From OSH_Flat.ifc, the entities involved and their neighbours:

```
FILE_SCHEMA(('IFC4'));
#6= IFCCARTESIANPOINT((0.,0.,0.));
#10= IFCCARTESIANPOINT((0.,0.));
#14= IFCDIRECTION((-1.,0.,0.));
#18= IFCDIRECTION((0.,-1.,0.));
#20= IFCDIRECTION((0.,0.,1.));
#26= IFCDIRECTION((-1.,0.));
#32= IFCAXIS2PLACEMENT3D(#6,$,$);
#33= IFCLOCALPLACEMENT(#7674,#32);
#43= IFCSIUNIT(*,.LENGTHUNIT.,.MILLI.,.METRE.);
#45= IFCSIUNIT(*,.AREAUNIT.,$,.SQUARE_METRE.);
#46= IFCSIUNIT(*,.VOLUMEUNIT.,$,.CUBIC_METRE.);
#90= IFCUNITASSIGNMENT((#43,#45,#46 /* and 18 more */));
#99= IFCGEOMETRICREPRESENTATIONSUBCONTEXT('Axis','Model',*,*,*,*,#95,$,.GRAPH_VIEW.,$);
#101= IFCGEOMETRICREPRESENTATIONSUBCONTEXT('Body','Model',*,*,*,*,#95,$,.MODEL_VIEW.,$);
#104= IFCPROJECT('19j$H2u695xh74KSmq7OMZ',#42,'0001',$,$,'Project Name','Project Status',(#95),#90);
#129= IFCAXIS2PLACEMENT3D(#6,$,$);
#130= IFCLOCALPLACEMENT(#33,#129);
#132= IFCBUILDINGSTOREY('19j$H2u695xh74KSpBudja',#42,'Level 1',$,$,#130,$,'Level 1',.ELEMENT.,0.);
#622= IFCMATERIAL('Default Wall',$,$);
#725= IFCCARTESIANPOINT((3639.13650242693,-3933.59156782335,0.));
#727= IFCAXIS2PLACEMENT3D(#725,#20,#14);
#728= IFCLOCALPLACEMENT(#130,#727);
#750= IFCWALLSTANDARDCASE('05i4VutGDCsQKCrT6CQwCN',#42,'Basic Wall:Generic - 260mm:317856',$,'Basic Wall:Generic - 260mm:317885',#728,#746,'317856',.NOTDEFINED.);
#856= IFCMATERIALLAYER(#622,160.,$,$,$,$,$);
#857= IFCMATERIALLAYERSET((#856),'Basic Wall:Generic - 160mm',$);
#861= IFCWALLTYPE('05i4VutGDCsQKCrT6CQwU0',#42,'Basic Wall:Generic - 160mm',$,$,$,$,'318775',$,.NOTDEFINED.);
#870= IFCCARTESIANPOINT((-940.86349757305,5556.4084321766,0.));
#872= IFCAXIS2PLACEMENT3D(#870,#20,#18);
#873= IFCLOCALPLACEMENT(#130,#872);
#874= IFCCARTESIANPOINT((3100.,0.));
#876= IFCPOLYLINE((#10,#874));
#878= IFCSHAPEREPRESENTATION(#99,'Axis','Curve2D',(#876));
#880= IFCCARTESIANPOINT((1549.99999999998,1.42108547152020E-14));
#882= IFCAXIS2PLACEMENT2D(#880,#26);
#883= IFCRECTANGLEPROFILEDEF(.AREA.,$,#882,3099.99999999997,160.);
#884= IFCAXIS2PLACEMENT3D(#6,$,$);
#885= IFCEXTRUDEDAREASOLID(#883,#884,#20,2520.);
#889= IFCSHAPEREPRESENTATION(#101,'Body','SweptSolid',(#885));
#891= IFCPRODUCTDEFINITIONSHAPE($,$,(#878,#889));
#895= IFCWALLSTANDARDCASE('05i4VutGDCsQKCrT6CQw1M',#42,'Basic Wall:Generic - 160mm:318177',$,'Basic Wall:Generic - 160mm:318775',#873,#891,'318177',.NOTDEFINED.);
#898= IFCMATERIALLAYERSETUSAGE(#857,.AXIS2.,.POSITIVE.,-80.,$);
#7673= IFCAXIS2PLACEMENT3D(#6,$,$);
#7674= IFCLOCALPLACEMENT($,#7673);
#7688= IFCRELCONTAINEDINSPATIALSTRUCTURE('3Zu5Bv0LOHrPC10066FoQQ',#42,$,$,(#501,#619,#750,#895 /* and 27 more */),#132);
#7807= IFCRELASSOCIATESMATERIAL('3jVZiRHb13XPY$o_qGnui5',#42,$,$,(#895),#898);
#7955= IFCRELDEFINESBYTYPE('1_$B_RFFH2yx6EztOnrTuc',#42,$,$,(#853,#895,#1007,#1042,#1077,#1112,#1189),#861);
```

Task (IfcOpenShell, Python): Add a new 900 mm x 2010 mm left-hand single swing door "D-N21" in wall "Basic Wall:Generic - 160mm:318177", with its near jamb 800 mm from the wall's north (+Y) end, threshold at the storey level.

```python
import numpy as np
import ifcopenshell
import ifcopenshell.api.feature
import ifcopenshell.api.geometry
import ifcopenshell.api.root
import ifcopenshell.api.spatial
import ifcopenshell.geom
import ifcopenshell.util.element
import ifcopenshell.util.placement
import ifcopenshell.util.representation
import ifcopenshell.util.shape
import ifcopenshell.util.unit

model = ifcopenshell.open("OSH_Flat.ifc")
unit_scale = ifcopenshell.util.unit.calculate_unit_scale(model)
settings = ifcopenshell.geom.settings()


def volume(element):
    """Net volume in cubic metres, openings subtracted."""
    shape = ifcopenshell.geom.create_shape(settings, element)
    return ifcopenshell.util.shape.get_volume(shape.geometry)


wall = model.by_guid("05i4VutGDCsQKCrT6CQw1M")
storey = ifcopenshell.util.element.get_container(wall, ifc_class="IfcBuildingStorey")
context = ifcopenshell.util.representation.get_context(model, "Model", "Body", "MODEL_VIEW")
before = volume(wall)

width, height, from_end, sill = 0.9, 2.01, 0.8, 0.0  # metres

# The wall runs along its own X axis, and the end named is its -X end.
wall_shape = ifcopenshell.geom.create_shape(settings, wall)
x, y, z = ifcopenshell.util.shape.get_vertices(wall_shape.geometry).T
start = x.min() + from_end
face, thickness = float(y.min()), float(y.max() - y.min())
wall_matrix = ifcopenshell.util.placement.get_local_placement(wall.ObjectPlacement)
level = ifcopenshell.util.placement.get_local_placement(storey.ObjectPlacement)[2, 3]


def in_wall(x, y):
    """Placement at x, y metres in the wall's axes, at sill height."""
    matrix = wall_matrix.copy()
    matrix[:, 3] = wall_matrix @ np.array([x / unit_scale, y / unit_scale, 0.0, 1.0])
    matrix[2, 3] = level + sill / unit_scale
    return matrix


# Opening: a box that overshoots both wall faces by 50 mm.
opening = ifcopenshell.api.root.create_entity(model, ifc_class="IfcOpeningElement", predefined_type="OPENING")
box = ifcopenshell.api.geometry.add_wall_representation(
    model, context=context, length=width, height=height, thickness=thickness + 0.1
)
ifcopenshell.api.geometry.assign_representation(model, product=opening, representation=box)
ifcopenshell.api.geometry.edit_object_placement(model, product=opening, matrix=in_wall(start, face - 0.05), is_si=False)
ifcopenshell.api.feature.add_feature(model, feature=opening, element=wall)

door = ifcopenshell.api.root.create_entity(model, ifc_class="IfcDoor", name="D-N21", predefined_type="DOOR")
door.OverallWidth, door.OverallHeight = width / unit_scale, height / unit_scale
door.OperationType = "SINGLE_SWING_LEFT"
body = ifcopenshell.api.geometry.add_door_representation(
    model,
    context=context,
    overall_width=door.OverallWidth,
    overall_height=door.OverallHeight,
    operation_type="SINGLE_SWING_LEFT",
    lining_properties={"LiningDepth": thickness / unit_scale, "ThresholdDepth": thickness / unit_scale},
)
ifcopenshell.api.geometry.assign_representation(model, product=door, representation=body)
ifcopenshell.api.spatial.assign_container(model, products=[door], relating_structure=storey)
ifcopenshell.api.feature.add_filling(model, opening=opening, element=door)

# The lining spans the wall, so the door starts at the wall face.
ifcopenshell.api.geometry.edit_object_placement(model, product=door, matrix=in_wall(start, face), is_si=False)

after = volume(wall)

print(f"wall volume {before:.3f} -> {after:.3f} m3")

model.write("OSH_Flat_updated.ifc")
```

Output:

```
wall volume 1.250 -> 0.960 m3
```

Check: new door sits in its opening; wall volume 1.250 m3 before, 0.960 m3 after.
